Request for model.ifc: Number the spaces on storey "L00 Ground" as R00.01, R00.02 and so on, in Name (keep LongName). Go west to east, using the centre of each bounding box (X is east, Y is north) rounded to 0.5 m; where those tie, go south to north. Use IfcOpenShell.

First a look at what the model holds.

```python
import ifcopenshell
import ifcopenshell.util.element
import ifcopenshell.util.placement

model = ifcopenshell.open("model.ifc")
print(model.schema)
storey = next(s for s in model.by_type("IfcBuildingStorey") if s.Name == "L00 Ground")
spaces = [e for e in ifcopenshell.util.element.get_decomposition(storey) if e.is_a("IfcSpace")]
for e in sorted(spaces, key=lambda e: e.id()):
    origin = ifcopenshell.util.placement.get_local_placement(e.ObjectPlacement)[:3, 3]
    print(e.id(), e.Name, e.LongName, origin.round(2) + 0.0, sep=" | ")
```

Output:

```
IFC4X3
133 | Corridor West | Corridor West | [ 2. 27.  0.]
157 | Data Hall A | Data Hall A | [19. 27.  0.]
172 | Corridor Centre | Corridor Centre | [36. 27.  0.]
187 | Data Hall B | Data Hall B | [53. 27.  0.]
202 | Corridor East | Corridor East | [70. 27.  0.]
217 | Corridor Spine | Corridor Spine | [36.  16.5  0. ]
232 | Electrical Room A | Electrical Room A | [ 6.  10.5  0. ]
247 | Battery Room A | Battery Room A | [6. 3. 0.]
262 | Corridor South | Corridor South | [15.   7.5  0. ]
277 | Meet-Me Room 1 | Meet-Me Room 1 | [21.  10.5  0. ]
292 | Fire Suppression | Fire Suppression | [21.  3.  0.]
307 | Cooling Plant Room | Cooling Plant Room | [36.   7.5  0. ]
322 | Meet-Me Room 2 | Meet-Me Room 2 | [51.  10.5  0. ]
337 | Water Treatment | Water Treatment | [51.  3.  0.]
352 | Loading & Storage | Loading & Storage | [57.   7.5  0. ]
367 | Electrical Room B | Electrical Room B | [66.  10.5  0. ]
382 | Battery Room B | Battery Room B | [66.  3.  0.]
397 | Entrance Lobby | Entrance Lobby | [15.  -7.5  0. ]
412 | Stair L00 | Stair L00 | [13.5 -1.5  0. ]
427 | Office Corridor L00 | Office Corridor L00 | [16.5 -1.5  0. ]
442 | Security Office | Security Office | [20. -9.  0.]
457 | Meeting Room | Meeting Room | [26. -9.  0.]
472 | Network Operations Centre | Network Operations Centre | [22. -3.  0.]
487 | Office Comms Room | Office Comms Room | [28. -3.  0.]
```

```python
import ifcopenshell
import ifcopenshell.geom
import ifcopenshell.util.element
import ifcopenshell.util.shape

model = ifcopenshell.open("model.ifc")
settings = ifcopenshell.geom.settings()
settings.set("use-world-coords", True)


def centre(element):
    shape = ifcopenshell.geom.create_shape(settings, element)
    return ifcopenshell.util.shape.get_bbox_centroid(shape.geometry)


storey = next(s for s in model.by_type("IfcBuildingStorey") if s.Name == "L00 Ground")
spaces = [e for e in ifcopenshell.util.element.get_decomposition(storey) if e.is_a("IfcSpace")]

# Insertion points can sit at a corner or the storey origin, so sort by the geometry (in metres).
centres = {e: centre(e) for e in spaces}
spaces.sort(key=lambda e: (round(centres[e][0] / 0.5), centres[e][1]))

for i, e in enumerate(spaces, start=1):
    number = f"R00.{i:02d}"
    e.Name = number
    print(e.id(), number)

model.write("model-out.ifc")
```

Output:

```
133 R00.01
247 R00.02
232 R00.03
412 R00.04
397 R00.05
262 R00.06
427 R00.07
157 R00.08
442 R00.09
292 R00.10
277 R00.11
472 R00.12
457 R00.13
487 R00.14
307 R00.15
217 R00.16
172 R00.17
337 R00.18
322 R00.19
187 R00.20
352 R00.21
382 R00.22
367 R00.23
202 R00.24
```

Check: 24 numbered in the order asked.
